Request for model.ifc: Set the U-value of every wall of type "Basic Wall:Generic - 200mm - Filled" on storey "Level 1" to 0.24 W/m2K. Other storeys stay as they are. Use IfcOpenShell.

First a look at what the model holds.

```python
import ifcopenshell
import ifcopenshell.util.element

model = ifcopenshell.open("model.ifc")
print(model.schema)
storey = next(s for s in model.by_type("IfcBuildingStorey") if s.Name == "Level 1")
walls = [e for e in ifcopenshell.util.element.get_decomposition(storey) if e.is_a("IfcWall")]
seen = {}
for e in walls:
    element_type = ifcopenshell.util.element.get_type(e)
    key = (element_type.Name if element_type != e and element_type else None, ifcopenshell.util.element.get_pset(e, "Pset_WallCommon", "ThermalTransmittance"))
    seen[key] = seen.get(key, 0) + 1
for (name, value), count in sorted(seen.items(), key=str):
    print(count, "x", name, "|", value)
```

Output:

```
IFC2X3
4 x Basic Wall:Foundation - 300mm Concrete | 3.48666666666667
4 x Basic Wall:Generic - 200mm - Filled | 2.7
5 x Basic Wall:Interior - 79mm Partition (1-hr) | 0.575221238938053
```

```python
import ifcopenshell
import ifcopenshell.api.pset
import ifcopenshell.util.element

model = ifcopenshell.open("model.ifc")

storey = next(s for s in model.by_type("IfcBuildingStorey") if s.Name == "Level 1")
walls = [e for e in ifcopenshell.util.element.get_decomposition(storey) if e.is_a("IfcWall")]

count = 0
for e in walls:
    element_type = ifcopenshell.util.element.get_type(e)
    if element_type in (None, e) or element_type.Name != "Basic Wall:Generic - 200mm - Filled":
        continue
    # add_pset returns the element's existing set when there is one.
    pset = ifcopenshell.api.pset.add_pset(model, product=e, name="Pset_WallCommon")
    ifcopenshell.api.pset.edit_pset(model, pset=pset, properties={"ThermalTransmittance": 0.24})
    count += 1

print(count, "walls updated")

model.write("model_rev.ifc")
```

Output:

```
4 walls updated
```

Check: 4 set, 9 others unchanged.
